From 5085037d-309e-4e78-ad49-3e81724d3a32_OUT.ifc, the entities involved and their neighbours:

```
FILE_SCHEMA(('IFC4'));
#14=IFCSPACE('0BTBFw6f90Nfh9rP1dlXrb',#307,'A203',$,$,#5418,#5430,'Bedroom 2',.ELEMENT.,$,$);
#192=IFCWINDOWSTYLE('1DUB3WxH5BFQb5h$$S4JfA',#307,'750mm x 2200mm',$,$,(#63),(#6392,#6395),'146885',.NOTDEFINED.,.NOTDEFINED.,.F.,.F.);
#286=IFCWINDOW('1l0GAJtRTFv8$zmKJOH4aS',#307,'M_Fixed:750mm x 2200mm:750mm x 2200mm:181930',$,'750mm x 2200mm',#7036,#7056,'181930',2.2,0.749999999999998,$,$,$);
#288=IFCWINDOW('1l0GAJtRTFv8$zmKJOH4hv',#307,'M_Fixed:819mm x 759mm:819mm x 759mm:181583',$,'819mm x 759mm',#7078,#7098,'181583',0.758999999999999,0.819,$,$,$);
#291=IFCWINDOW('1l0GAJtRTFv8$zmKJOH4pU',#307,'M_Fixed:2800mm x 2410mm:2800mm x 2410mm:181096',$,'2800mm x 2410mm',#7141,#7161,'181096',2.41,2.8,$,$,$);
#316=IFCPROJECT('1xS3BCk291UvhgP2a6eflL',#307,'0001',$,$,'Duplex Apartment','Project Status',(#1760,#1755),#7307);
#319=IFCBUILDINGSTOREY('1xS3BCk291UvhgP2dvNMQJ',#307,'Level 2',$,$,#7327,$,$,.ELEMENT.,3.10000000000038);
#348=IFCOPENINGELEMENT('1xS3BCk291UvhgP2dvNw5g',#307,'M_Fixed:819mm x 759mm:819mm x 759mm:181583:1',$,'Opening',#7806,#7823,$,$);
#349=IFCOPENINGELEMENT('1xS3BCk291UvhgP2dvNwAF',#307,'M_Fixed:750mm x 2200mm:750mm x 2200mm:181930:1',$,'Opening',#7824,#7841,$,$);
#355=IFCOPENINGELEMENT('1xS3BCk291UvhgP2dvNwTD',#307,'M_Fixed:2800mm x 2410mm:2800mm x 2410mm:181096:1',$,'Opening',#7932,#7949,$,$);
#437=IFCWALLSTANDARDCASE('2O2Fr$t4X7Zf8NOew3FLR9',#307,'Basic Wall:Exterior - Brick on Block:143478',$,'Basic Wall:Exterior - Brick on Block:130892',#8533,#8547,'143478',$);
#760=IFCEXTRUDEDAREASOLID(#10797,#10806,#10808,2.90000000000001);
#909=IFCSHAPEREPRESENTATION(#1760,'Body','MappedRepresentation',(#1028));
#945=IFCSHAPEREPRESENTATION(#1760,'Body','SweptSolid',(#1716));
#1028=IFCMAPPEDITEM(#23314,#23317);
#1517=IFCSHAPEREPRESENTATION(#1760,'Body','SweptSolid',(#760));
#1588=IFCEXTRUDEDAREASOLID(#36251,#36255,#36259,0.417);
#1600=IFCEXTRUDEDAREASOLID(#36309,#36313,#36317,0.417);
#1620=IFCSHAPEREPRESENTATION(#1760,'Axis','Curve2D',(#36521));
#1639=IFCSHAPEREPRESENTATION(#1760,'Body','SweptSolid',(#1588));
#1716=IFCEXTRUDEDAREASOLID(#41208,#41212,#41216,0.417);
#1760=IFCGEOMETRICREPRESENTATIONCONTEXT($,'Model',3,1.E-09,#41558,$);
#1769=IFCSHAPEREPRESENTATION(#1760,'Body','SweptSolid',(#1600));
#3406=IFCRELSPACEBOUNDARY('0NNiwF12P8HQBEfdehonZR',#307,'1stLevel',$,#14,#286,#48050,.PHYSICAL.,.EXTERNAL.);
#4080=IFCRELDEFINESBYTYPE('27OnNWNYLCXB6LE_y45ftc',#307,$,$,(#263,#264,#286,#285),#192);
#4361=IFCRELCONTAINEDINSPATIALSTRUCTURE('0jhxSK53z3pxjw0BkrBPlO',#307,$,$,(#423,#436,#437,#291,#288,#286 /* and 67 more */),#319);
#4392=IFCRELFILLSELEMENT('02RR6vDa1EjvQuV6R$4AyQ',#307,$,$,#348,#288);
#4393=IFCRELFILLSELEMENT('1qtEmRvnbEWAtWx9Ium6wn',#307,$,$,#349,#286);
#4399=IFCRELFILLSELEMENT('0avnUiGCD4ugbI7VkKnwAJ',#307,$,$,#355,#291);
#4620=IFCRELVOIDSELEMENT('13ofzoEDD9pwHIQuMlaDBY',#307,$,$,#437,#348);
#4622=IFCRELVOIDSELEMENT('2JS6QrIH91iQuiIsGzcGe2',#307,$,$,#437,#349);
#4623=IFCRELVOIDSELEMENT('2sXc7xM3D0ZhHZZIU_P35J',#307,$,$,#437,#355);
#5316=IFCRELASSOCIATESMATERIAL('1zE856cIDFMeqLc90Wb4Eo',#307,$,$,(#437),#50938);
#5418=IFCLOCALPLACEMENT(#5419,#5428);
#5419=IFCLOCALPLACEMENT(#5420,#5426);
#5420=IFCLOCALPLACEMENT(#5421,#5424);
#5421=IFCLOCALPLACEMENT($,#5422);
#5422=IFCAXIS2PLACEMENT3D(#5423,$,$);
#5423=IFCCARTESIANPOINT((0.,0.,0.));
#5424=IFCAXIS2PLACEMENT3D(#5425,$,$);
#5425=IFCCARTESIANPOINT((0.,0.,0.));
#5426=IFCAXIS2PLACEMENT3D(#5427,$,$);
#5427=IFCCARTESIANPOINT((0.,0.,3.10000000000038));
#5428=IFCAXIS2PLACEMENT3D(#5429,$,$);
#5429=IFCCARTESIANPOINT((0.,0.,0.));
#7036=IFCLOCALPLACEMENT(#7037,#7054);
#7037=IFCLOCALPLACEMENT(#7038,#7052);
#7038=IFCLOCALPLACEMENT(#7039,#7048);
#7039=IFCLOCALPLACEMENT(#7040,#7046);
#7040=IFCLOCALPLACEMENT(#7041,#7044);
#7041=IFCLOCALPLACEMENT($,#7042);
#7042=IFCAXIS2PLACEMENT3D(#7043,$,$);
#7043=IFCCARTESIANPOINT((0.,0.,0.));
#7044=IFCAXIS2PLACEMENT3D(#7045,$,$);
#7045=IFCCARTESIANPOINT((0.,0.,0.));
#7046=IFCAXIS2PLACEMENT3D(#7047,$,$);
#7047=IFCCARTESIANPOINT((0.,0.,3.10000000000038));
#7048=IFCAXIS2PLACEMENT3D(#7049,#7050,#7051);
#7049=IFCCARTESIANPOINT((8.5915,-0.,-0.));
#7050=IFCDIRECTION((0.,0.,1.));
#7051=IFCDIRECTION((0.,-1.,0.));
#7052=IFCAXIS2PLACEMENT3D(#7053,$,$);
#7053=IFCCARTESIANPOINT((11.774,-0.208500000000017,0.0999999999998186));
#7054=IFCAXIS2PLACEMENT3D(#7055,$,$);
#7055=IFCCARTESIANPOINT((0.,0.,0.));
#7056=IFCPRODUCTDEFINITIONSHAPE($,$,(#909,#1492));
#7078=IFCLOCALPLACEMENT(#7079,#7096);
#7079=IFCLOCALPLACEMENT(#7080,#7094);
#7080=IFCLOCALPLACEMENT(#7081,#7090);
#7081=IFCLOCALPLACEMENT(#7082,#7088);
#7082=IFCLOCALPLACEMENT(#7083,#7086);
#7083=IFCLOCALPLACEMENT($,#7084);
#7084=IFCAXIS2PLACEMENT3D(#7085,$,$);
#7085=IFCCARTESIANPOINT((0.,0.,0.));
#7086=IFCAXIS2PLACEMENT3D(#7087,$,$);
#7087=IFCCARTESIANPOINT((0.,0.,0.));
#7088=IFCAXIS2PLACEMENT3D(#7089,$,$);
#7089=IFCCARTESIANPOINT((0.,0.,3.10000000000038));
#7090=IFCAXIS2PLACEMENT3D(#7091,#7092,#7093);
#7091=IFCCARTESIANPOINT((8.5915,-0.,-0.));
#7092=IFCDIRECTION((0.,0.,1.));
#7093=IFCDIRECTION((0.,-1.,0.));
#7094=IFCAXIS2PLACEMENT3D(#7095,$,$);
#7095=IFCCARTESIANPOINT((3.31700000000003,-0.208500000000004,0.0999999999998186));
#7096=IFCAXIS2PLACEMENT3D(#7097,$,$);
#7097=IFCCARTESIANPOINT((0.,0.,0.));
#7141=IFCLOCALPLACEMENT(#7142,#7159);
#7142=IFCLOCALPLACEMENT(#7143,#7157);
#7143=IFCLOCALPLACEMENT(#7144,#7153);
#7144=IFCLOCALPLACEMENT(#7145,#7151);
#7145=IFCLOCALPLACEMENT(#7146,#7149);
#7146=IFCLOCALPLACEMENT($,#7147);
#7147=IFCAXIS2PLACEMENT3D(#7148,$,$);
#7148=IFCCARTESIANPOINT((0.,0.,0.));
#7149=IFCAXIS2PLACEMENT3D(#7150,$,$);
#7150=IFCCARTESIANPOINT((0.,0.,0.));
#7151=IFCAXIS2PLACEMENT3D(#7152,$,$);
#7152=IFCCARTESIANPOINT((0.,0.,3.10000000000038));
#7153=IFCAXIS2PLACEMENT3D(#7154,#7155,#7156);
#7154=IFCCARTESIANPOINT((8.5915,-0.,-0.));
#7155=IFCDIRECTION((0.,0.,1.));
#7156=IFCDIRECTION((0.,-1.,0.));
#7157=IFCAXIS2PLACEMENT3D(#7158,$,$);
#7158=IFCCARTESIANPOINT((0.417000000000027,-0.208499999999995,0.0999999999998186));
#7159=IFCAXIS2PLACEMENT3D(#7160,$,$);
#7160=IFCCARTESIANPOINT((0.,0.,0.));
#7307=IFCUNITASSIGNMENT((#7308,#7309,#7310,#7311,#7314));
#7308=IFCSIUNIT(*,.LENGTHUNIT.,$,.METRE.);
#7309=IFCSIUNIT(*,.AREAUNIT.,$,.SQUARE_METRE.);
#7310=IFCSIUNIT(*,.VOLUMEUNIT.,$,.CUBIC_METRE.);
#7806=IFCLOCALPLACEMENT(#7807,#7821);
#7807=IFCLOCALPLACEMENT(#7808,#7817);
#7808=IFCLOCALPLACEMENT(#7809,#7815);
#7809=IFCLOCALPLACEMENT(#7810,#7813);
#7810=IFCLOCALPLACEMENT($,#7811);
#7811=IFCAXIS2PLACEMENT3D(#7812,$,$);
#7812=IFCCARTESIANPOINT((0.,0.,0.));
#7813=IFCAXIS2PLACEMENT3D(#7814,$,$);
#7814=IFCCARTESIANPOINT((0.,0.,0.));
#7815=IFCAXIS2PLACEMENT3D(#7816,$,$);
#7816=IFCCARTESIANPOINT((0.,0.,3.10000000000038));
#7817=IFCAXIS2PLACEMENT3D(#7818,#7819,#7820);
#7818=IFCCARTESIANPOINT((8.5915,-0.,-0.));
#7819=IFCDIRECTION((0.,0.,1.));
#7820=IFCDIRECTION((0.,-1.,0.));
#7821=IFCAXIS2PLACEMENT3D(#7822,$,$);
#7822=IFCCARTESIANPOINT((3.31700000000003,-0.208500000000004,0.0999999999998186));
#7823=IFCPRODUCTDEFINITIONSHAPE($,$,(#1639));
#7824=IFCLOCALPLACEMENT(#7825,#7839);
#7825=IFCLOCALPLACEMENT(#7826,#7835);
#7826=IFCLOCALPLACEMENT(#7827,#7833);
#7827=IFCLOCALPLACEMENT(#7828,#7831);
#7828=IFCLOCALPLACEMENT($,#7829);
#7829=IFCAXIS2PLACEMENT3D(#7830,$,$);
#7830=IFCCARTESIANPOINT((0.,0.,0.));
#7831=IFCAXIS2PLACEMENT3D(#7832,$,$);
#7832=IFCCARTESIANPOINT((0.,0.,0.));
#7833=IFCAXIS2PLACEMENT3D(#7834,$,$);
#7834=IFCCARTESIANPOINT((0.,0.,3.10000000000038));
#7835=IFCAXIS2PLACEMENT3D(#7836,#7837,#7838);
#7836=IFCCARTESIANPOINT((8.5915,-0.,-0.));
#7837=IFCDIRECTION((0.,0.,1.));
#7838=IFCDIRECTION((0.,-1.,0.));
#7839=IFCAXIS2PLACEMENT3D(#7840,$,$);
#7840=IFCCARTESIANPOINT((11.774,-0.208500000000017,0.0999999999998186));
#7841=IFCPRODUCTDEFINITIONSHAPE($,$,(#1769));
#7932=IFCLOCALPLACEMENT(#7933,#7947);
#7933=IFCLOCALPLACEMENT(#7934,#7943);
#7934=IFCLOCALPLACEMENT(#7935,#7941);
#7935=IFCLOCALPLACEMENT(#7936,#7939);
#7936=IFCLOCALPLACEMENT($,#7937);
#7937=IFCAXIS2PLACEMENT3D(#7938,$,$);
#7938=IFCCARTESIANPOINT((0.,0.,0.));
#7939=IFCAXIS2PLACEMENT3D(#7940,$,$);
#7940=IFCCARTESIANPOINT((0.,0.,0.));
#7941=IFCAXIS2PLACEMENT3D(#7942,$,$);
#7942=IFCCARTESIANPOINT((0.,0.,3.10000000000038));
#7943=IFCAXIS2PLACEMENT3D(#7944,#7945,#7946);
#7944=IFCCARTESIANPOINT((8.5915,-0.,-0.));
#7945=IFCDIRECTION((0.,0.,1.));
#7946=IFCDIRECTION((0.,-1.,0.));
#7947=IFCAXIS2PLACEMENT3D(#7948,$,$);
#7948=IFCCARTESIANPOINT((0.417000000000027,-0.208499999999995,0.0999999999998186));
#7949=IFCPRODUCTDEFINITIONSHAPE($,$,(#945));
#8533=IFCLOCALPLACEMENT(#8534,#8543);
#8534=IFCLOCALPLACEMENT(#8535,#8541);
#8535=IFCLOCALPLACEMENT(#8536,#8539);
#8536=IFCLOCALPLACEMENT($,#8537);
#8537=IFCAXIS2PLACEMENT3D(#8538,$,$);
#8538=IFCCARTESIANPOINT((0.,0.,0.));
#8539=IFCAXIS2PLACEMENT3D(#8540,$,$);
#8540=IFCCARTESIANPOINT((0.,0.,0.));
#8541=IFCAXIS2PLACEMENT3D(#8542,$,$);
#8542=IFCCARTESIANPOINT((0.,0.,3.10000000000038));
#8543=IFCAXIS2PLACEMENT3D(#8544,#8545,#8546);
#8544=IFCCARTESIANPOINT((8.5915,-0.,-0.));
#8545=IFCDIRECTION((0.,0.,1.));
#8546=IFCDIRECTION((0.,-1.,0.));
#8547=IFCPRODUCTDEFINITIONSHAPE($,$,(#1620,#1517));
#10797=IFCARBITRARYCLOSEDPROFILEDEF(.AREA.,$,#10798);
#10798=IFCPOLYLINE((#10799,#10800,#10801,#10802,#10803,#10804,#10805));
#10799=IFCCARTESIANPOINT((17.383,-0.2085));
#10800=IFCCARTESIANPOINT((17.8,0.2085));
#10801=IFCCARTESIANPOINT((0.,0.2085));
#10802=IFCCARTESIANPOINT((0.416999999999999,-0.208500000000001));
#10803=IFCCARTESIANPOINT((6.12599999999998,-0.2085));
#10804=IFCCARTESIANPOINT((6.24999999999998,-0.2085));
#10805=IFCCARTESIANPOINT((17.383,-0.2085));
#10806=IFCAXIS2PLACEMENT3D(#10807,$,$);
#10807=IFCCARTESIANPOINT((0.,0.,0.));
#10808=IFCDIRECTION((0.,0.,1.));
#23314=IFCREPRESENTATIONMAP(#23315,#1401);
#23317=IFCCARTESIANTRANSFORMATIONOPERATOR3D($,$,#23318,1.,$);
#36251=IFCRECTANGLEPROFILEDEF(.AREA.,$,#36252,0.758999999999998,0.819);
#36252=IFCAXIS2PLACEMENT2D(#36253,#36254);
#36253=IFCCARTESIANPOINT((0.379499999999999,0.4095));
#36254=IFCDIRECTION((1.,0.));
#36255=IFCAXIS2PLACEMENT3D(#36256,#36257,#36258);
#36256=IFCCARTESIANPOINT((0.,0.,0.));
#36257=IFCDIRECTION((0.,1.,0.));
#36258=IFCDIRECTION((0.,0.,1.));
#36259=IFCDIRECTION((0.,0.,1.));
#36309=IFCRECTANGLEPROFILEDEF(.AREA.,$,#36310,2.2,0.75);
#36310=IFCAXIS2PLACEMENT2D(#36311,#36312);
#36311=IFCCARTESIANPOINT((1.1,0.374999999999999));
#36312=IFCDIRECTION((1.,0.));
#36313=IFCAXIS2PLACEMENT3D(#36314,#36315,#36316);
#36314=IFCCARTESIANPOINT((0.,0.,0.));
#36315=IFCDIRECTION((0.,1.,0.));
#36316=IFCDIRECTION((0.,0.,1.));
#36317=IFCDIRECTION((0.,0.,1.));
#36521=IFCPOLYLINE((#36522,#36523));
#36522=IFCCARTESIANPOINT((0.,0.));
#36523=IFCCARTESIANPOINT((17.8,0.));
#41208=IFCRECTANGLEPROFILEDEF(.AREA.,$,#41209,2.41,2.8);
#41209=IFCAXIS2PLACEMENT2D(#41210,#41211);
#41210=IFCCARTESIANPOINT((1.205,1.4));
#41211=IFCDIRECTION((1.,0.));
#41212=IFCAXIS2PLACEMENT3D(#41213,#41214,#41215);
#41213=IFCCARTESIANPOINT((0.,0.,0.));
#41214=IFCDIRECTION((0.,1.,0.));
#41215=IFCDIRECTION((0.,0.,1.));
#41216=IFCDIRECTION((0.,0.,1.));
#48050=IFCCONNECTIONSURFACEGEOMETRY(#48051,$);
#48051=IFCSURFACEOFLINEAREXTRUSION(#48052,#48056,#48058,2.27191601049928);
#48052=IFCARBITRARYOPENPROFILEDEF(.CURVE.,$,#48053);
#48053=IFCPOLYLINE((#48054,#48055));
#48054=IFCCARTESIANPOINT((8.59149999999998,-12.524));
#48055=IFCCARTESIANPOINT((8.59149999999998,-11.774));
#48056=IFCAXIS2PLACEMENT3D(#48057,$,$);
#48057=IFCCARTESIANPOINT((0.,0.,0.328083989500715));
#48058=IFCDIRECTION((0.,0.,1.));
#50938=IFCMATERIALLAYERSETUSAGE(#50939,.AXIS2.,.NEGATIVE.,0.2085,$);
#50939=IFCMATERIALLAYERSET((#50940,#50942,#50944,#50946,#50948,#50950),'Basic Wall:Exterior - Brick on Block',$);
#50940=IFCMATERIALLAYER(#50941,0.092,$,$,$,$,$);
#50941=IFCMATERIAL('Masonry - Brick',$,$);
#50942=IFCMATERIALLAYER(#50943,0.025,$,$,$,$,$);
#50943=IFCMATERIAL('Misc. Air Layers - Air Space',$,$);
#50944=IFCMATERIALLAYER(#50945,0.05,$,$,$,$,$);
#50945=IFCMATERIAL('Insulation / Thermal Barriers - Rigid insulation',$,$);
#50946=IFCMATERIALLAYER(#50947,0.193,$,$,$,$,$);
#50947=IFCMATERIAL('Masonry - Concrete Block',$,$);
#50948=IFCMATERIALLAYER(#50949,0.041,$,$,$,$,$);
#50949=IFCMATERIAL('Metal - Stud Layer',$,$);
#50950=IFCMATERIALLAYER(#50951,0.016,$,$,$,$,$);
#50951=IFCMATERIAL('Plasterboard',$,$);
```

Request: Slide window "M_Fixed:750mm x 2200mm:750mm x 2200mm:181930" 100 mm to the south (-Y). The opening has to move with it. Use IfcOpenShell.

```python
import numpy as np
import ifcopenshell
import ifcopenshell.api.geometry
import ifcopenshell.util.placement

model = ifcopenshell.open("5085037d-309e-4e78-ad49-3e81724d3a32_OUT.ifc")

window = model.by_guid("1l0GAJtRTFv8$zmKJOH4aS")
opening = window.FillsVoids[0].RelatingOpeningElement
wall = opening.VoidsElements[0].RelatingBuildingElement

wall_matrix = ifcopenshell.util.placement.get_local_placement(wall.ObjectPlacement)
shift = wall_matrix[:3, 0] * 0.1
before = ifcopenshell.util.placement.get_local_placement(window.ObjectPlacement)[:3, 3].copy()

# The window is not placed relative to its opening, so move both.
for product in (opening, window):
    matrix = ifcopenshell.util.placement.get_local_placement(product.ObjectPlacement)
    matrix[:3, 3] += shift
    ifcopenshell.api.geometry.edit_object_placement(model, product=product, matrix=matrix, is_si=False)

# Space boundary surfaces are stored in each space's coordinates; move them too.
for rel in window.ProvidesBoundaries:
    if not rel.ConnectionGeometry:
        continue
    surface = rel.ConnectionGeometry.SurfaceOnRelatingElement
    space_matrix = ifcopenshell.util.placement.get_local_placement(rel.RelatingSpace.ObjectPlacement)
    point = np.array(surface.Position.Location.Coordinates) + space_matrix[:3, :3].T @ shift
    surface.Position = model.createIfcAxis2Placement3D(
        model.createIfcCartesianPoint(point.tolist()), surface.Position.Axis, surface.Position.RefDirection
    )

after = ifcopenshell.util.placement.get_local_placement(window.ObjectPlacement)[:3, 3]
print("window moved by", (after - before).round(3) + 0.0)

model.write("5085037d-309e-4e78-ad49-3e81724d3a32_OUT_updated.ifc")
```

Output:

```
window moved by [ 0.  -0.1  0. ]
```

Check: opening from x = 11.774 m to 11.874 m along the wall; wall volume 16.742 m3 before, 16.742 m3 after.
